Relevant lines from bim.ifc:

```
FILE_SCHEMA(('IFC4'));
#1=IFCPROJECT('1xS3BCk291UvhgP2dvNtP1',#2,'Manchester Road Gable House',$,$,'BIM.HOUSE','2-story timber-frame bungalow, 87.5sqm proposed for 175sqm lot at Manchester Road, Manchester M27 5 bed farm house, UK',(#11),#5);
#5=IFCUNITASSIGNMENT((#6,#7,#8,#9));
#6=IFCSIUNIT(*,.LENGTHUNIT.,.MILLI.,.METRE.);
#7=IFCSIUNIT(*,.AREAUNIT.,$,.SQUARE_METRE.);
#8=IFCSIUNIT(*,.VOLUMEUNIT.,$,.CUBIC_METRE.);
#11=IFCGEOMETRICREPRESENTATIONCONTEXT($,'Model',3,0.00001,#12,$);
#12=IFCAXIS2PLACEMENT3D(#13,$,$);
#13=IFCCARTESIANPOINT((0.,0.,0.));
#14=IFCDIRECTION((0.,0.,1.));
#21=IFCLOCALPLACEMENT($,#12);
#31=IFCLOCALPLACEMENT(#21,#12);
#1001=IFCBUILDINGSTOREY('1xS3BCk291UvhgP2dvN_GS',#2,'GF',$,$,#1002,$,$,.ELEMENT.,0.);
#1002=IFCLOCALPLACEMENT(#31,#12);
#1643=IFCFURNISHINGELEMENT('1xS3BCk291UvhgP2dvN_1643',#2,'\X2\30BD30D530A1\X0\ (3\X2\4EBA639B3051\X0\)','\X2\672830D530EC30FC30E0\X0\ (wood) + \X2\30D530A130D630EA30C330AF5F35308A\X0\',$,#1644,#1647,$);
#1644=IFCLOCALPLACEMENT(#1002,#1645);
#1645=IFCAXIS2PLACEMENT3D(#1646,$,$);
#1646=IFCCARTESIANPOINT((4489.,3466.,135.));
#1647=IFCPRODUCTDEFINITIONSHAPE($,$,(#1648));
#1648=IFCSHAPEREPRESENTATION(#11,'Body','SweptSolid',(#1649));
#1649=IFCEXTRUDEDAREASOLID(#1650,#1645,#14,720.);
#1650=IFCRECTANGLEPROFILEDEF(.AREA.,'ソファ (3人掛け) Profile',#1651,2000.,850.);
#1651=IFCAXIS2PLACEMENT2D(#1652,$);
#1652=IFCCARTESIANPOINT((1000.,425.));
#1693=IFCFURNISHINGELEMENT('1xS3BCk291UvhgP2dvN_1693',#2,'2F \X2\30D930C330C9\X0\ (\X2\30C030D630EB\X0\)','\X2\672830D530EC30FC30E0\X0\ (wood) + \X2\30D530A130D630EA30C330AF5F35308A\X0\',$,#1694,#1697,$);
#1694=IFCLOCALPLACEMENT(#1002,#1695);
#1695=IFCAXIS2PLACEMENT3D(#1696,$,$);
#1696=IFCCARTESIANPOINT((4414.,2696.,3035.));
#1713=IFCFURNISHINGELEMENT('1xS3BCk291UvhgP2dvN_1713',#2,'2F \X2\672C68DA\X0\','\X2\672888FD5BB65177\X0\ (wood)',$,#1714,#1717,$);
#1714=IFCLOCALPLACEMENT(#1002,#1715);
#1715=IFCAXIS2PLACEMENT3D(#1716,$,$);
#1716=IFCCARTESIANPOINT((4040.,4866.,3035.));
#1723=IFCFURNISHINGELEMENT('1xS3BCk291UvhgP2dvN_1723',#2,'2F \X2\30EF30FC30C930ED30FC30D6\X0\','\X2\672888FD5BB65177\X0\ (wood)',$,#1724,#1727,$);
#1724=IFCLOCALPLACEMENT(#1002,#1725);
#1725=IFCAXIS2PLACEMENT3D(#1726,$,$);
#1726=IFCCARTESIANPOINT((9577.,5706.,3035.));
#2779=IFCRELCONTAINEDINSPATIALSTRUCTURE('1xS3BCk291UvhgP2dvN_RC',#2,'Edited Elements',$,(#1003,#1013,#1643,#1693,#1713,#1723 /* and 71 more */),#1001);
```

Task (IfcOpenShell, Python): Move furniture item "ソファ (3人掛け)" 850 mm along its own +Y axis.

```python
import ifcopenshell
import ifcopenshell.api.geometry
import ifcopenshell.util.placement
import ifcopenshell.util.unit

model = ifcopenshell.open("bim.ifc")
unit_scale = ifcopenshell.util.unit.calculate_unit_scale(model)

item = model.by_guid("1xS3BCk291UvhgP2dvN_1643")
matrix = ifcopenshell.util.placement.get_local_placement(item.ObjectPlacement)
matrix[:3, 3] += matrix[:3, 1] * 0.85 / unit_scale
ifcopenshell.api.geometry.edit_object_placement(model, product=item, matrix=matrix, is_si=False)

print(ifcopenshell.util.placement.get_local_placement(item.ObjectPlacement).round(3) + 0.0)

model.write("bim_edited.ifc")
```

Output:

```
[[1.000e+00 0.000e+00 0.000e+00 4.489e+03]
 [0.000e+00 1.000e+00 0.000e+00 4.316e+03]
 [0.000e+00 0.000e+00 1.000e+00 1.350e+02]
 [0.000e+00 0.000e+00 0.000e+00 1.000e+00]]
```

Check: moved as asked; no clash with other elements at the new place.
